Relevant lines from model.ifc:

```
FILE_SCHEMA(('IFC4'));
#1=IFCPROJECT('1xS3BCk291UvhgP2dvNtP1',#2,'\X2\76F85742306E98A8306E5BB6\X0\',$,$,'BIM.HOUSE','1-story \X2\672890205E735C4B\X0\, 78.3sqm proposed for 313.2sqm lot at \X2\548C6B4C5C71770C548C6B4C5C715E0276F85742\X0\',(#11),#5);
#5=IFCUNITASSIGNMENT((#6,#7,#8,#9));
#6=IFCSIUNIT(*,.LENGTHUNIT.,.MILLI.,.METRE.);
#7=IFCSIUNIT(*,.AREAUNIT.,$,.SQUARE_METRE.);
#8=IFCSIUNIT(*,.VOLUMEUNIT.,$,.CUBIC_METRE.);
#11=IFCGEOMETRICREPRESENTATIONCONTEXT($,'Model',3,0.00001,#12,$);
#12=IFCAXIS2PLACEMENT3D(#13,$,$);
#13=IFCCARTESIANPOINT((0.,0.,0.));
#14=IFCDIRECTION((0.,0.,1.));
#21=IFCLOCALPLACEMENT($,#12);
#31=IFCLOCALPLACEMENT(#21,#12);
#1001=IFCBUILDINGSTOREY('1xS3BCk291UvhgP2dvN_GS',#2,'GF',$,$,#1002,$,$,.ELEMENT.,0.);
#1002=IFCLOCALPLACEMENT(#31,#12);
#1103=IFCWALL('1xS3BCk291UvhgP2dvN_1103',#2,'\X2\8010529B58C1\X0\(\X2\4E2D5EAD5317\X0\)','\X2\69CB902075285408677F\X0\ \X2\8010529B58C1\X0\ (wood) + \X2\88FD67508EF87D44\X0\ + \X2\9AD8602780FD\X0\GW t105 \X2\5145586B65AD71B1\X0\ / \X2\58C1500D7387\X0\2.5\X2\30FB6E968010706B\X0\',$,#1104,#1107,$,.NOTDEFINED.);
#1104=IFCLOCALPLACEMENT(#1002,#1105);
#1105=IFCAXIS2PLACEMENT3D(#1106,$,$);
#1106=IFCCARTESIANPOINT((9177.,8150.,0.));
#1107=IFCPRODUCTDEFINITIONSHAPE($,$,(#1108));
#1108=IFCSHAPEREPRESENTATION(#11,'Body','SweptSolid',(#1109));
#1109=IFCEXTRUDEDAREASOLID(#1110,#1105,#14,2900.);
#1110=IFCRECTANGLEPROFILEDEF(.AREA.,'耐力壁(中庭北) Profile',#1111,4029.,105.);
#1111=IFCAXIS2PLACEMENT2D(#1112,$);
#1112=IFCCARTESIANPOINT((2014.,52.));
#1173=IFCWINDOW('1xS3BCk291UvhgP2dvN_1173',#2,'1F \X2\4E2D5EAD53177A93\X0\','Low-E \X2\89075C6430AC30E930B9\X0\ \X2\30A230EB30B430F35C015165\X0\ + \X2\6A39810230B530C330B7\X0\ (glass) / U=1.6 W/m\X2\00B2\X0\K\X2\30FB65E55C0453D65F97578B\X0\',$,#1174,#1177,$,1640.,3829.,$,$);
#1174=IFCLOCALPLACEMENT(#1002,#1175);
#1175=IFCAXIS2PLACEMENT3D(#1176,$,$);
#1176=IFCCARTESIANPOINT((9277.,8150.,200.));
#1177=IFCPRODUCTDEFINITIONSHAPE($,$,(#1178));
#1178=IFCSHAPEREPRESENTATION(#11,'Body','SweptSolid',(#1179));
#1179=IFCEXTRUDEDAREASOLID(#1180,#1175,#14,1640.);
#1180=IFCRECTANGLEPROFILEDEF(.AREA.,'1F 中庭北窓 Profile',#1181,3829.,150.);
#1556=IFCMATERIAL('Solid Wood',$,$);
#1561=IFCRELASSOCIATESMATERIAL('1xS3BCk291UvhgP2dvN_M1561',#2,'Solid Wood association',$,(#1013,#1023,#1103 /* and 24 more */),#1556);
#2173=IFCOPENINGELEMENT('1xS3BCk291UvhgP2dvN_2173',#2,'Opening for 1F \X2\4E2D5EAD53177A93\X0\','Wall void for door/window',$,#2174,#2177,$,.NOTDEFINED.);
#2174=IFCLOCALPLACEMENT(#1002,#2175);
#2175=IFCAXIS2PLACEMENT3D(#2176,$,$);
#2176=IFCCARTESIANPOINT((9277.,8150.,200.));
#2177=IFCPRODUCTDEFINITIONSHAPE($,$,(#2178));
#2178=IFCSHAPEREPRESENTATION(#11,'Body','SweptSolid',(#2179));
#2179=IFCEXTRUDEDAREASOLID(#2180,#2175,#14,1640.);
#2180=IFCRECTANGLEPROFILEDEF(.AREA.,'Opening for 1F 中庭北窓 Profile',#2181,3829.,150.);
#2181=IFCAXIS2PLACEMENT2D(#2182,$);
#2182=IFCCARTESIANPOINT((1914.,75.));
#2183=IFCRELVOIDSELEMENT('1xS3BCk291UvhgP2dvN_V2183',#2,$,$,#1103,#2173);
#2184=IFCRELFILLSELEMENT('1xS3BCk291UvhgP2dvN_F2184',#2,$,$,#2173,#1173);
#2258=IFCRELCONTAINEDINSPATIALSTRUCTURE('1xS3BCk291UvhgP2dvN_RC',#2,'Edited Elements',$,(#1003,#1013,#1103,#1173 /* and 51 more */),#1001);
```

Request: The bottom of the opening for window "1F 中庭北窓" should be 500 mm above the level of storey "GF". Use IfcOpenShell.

```python
import numpy as np
import ifcopenshell
import ifcopenshell.api.geometry
import ifcopenshell.geom
import ifcopenshell.util.element
import ifcopenshell.util.placement
import ifcopenshell.util.shape
import ifcopenshell.util.unit

model = ifcopenshell.open("model.ifc")
unit_scale = ifcopenshell.util.unit.calculate_unit_scale(model)

window = model.by_id(1173)
opening = window.FillsVoids[0].RelatingOpeningElement
storey = ifcopenshell.util.element.get_container(window, ifc_class="IfcBuildingStorey")
level = ifcopenshell.util.placement.get_local_placement(storey.ObjectPlacement)[2, 3]

# The opening's origin need not be at the sill, so measure its lowest point.
shape = ifcopenshell.geom.create_shape(ifcopenshell.geom.settings(), opening)
bottom = ifcopenshell.util.shape.get_shape_bottom_elevation(shape, shape.geometry) / unit_scale
dz = level + 0.5 / unit_scale - bottom

shift = np.array([0.0, 0.0, dz])
# The window is not placed relative to its opening, so move both.
for product in (opening, window):
    matrix = ifcopenshell.util.placement.get_local_placement(product.ObjectPlacement)
    matrix[:3, 3] += shift
    ifcopenshell.api.geometry.edit_object_placement(model, product=product, matrix=matrix, is_si=False)

print(f"moved by {dz * unit_scale:+.3f} m")

model.write("model_updated.ifc")
```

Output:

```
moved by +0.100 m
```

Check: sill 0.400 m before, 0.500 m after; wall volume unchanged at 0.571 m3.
